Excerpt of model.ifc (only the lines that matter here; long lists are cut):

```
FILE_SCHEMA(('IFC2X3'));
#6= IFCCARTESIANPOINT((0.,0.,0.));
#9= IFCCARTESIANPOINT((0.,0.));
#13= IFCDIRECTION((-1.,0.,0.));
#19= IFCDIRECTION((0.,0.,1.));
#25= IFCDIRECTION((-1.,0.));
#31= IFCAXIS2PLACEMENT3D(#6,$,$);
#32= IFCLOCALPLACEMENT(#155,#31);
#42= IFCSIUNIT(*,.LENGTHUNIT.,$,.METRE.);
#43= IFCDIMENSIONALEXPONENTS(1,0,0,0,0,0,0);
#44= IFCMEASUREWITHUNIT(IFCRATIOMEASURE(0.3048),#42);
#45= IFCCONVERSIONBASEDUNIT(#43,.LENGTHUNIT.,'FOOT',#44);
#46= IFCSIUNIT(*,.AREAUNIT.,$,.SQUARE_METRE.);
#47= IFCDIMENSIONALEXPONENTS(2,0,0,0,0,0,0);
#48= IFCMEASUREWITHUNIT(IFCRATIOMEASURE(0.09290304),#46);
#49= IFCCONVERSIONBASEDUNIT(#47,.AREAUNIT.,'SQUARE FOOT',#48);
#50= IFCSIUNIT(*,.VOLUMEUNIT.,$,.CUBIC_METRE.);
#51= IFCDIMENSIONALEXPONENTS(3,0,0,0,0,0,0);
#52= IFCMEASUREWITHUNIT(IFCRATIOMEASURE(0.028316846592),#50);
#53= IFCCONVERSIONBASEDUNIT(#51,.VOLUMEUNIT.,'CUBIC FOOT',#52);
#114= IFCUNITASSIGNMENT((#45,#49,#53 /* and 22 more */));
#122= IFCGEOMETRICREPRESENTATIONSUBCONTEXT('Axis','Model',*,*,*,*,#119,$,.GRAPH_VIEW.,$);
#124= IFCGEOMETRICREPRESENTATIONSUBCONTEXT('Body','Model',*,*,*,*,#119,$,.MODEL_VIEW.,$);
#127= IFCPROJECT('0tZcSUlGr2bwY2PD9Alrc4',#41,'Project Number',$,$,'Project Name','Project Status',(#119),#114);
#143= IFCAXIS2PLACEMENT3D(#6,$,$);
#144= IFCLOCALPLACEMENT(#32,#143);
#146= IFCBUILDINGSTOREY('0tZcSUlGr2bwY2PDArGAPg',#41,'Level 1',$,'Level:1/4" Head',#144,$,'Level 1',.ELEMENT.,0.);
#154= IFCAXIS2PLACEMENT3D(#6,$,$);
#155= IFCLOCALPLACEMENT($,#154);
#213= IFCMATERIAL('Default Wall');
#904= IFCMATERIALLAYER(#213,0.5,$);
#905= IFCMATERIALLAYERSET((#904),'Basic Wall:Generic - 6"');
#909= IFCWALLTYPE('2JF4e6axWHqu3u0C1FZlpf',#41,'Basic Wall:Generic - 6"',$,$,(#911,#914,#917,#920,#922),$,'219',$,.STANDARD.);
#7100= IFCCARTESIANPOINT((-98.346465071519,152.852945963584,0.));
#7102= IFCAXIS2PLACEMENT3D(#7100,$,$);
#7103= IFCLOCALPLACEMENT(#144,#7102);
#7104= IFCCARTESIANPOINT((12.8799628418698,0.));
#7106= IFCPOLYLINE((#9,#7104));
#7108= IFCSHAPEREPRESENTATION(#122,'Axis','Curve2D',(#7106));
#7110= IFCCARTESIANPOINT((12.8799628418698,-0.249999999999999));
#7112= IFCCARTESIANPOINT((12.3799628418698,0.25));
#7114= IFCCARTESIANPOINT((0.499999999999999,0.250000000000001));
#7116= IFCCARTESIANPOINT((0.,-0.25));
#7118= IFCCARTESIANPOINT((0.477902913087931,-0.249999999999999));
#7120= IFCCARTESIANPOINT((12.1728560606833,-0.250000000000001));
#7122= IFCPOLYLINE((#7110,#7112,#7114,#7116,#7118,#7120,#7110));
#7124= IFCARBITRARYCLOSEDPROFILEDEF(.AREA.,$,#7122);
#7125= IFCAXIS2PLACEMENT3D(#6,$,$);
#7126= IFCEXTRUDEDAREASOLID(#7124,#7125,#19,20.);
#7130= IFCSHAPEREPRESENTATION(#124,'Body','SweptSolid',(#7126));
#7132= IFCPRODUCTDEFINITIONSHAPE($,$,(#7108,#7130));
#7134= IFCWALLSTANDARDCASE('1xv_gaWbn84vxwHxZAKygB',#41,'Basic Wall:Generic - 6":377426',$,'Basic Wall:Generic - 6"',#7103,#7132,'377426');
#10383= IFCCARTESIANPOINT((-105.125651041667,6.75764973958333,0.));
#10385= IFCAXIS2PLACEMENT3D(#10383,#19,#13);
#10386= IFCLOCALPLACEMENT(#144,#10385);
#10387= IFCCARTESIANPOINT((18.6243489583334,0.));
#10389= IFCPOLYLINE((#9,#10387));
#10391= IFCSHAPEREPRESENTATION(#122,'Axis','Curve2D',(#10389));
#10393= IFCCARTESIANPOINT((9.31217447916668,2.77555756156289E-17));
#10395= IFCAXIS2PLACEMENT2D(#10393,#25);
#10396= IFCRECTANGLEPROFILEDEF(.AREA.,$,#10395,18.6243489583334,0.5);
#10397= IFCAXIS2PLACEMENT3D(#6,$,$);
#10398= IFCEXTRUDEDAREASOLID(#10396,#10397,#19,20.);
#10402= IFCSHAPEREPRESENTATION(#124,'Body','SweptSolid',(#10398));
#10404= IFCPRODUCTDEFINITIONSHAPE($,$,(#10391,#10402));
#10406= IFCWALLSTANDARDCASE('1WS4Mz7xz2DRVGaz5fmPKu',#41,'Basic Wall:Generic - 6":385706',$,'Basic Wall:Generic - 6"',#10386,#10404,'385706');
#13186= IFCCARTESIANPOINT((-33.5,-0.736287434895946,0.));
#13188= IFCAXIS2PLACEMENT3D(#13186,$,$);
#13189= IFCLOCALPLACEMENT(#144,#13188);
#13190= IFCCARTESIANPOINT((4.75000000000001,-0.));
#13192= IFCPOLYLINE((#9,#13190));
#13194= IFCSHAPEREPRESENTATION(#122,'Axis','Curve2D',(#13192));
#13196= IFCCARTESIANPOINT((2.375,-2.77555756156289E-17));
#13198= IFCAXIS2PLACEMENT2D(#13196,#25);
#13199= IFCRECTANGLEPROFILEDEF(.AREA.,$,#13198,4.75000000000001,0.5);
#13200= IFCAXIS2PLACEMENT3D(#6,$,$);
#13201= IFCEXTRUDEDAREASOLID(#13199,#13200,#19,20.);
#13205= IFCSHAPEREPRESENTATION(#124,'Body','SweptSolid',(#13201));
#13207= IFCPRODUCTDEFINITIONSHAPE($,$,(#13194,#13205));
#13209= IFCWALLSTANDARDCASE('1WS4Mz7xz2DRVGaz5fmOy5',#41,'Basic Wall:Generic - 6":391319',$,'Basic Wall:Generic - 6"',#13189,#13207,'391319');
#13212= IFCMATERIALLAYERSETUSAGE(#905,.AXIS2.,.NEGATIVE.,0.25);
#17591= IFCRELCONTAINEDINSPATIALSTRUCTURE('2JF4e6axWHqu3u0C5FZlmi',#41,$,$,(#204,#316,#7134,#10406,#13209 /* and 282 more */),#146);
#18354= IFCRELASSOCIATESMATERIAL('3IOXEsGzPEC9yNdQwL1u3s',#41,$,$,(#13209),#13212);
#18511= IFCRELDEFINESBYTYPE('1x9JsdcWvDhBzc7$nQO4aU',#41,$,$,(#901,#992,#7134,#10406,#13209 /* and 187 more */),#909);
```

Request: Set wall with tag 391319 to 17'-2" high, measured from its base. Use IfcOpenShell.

```python
import ifcopenshell
import ifcopenshell.geom
import ifcopenshell.util.representation
import ifcopenshell.util.shape
import ifcopenshell.util.unit

model = ifcopenshell.open("model.ifc")
unit_scale = ifcopenshell.util.unit.calculate_unit_scale(model)
settings = ifcopenshell.geom.settings()


def volume(element):
    """Net volume in cubic metres, openings subtracted."""
    shape = ifcopenshell.geom.create_shape(settings, element)
    return ifcopenshell.util.shape.get_volume(shape.geometry)


wall = model.by_guid("1WS4Mz7xz2DRVGaz5fmOy5")
before = volume(wall)

body = ifcopenshell.util.representation.get_representation(wall, "Model", "Body")
solid = body.Items[0]
old_height = solid.Depth
solid.Depth = 206 * 0.0254 / unit_scale
after = volume(wall)

print(f"height {old_height:g} -> {solid.Depth:g}, volume {before:.3f} -> {after:.3f} m3")

model.write("model-out.ifc")
```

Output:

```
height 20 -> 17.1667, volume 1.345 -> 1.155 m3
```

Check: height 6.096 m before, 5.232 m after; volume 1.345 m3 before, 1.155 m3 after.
